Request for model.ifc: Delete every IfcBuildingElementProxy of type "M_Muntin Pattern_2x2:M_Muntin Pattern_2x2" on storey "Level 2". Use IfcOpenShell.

First a look at what the model holds.

```python
import ifcopenshell
import ifcopenshell.util.element

model = ifcopenshell.open("model.ifc")
print(model.schema)
storey = next(s for s in model.by_type("IfcBuildingStorey") if s.Name == "Level 2")
proxies = [e for e in ifcopenshell.util.element.get_decomposition(storey) if e.is_a("IfcBuildingElementProxy")]
seen = {}
for e in proxies:
    element_type = ifcopenshell.util.element.get_type(e)
    name = element_type.Name if element_type not in (None, e) else None
    seen[name] = seen.get(name, 0) + 1
for name, count in sorted(seen.items(), key=str):
    print(count, "x", name)
```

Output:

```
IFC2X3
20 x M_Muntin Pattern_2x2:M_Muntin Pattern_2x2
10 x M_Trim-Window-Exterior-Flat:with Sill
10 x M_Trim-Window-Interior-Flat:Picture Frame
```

```python
import ifcopenshell
import ifcopenshell.api.root
import ifcopenshell.util.element

model = ifcopenshell.open("model.ifc")

storey = next(s for s in model.by_type("IfcBuildingStorey") if s.Name == "Level 2")
proxies = [e for e in ifcopenshell.util.element.get_decomposition(storey) if e.is_a("IfcBuildingElementProxy")]
targets = [e for e in proxies if (t := ifcopenshell.util.element.get_type(e)) not in (None, e) and t.Name == "M_Muntin Pattern_2x2:M_Muntin Pattern_2x2"]

for e in targets:
    ifcopenshell.api.root.remove_product(model, product=e)
print(len(targets), "removed")

model.write("model_edited.ifc")
```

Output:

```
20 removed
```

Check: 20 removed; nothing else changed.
